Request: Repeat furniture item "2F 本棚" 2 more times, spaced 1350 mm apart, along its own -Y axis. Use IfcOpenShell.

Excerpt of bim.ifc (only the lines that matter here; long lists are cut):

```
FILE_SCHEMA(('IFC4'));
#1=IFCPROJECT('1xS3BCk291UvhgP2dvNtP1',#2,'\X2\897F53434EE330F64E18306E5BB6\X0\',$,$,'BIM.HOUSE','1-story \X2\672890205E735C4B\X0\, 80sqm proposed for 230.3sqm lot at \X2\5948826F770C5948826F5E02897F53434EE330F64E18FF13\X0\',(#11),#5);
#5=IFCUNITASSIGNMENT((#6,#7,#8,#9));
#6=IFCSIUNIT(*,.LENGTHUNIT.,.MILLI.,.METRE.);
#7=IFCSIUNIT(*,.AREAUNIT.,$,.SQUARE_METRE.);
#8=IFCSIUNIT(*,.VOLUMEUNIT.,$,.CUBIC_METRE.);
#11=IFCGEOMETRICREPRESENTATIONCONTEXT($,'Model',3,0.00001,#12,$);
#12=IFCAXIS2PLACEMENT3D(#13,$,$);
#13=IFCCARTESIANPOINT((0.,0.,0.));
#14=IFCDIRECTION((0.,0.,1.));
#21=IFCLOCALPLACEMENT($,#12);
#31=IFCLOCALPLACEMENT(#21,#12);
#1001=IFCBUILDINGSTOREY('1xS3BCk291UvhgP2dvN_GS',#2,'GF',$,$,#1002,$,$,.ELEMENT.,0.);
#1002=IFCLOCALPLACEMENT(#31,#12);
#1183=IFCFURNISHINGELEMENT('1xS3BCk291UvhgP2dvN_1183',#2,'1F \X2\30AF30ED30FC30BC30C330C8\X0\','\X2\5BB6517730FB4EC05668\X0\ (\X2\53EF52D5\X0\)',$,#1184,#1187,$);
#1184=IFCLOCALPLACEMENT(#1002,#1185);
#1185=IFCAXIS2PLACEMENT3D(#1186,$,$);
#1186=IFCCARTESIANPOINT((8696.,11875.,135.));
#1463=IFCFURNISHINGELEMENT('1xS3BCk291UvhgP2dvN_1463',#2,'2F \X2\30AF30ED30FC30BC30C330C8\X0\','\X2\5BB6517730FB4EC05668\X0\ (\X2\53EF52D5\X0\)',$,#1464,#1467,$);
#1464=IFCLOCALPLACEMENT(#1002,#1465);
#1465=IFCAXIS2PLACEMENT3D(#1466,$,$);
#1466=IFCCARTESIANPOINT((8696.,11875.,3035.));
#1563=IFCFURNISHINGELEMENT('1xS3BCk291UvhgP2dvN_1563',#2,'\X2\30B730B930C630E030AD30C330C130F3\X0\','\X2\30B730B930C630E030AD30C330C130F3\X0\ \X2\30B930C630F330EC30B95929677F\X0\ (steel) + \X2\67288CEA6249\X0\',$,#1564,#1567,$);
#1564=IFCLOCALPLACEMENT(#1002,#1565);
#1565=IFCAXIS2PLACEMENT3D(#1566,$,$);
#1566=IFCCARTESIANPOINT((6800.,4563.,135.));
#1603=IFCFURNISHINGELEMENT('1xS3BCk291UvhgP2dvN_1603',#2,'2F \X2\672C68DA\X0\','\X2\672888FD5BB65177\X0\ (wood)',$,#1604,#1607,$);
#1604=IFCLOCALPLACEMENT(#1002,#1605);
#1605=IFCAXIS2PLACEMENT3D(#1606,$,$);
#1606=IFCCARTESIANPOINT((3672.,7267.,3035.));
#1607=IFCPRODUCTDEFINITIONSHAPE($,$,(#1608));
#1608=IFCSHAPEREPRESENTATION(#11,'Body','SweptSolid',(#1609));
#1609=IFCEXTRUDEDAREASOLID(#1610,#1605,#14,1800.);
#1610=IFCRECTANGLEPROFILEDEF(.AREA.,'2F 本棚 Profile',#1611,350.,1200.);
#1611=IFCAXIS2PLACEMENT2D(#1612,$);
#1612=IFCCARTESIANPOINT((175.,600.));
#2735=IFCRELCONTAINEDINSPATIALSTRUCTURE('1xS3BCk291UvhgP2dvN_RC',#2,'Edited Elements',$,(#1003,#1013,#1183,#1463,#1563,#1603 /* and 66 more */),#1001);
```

```python
import ifcopenshell
import ifcopenshell.api.geometry
import ifcopenshell.api.root
import ifcopenshell.util.element
import ifcopenshell.util.placement
import ifcopenshell.util.unit

model = ifcopenshell.open("bim.ifc")
unit_scale = ifcopenshell.util.unit.calculate_unit_scale(model)


def reuse_history(source, copy):
    """copy_class also copies each property set's owner history, people and application; keep the originals."""
    for rel in copy.IsDefinedBy:
        if rel.is_a("IfcRelDefinesByProperties") and (history := rel.RelatingPropertyDefinition.OwnerHistory):
            rel.RelatingPropertyDefinition.OwnerHistory = source.OwnerHistory
            ifcopenshell.util.element.remove_deep2(model, history)


source = model.by_guid("1xS3BCk291UvhgP2dvN_1603")
base = ifcopenshell.util.placement.get_local_placement(source.ObjectPlacement)
step = -base[:3, 1] * 1.35 / unit_scale

for i in range(1, 3):
    copy = ifcopenshell.api.root.copy_class(model, product=source)
    copy.Representation = ifcopenshell.util.element.copy_deep(
        model, source.Representation, exclude=["IfcGeometricRepresentationContext", "IfcRepresentationMap"]
    )
    reuse_history(source, copy)
    matrix = base.copy()
    matrix[:3, 3] += i * step
    print("added at", matrix[:3, 3].round(3) + 0.0)
    ifcopenshell.api.geometry.edit_object_placement(model, product=copy, matrix=matrix, is_si=False)

model.write("bim_rev.ifc")
```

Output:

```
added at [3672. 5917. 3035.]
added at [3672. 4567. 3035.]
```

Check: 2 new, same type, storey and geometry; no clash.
